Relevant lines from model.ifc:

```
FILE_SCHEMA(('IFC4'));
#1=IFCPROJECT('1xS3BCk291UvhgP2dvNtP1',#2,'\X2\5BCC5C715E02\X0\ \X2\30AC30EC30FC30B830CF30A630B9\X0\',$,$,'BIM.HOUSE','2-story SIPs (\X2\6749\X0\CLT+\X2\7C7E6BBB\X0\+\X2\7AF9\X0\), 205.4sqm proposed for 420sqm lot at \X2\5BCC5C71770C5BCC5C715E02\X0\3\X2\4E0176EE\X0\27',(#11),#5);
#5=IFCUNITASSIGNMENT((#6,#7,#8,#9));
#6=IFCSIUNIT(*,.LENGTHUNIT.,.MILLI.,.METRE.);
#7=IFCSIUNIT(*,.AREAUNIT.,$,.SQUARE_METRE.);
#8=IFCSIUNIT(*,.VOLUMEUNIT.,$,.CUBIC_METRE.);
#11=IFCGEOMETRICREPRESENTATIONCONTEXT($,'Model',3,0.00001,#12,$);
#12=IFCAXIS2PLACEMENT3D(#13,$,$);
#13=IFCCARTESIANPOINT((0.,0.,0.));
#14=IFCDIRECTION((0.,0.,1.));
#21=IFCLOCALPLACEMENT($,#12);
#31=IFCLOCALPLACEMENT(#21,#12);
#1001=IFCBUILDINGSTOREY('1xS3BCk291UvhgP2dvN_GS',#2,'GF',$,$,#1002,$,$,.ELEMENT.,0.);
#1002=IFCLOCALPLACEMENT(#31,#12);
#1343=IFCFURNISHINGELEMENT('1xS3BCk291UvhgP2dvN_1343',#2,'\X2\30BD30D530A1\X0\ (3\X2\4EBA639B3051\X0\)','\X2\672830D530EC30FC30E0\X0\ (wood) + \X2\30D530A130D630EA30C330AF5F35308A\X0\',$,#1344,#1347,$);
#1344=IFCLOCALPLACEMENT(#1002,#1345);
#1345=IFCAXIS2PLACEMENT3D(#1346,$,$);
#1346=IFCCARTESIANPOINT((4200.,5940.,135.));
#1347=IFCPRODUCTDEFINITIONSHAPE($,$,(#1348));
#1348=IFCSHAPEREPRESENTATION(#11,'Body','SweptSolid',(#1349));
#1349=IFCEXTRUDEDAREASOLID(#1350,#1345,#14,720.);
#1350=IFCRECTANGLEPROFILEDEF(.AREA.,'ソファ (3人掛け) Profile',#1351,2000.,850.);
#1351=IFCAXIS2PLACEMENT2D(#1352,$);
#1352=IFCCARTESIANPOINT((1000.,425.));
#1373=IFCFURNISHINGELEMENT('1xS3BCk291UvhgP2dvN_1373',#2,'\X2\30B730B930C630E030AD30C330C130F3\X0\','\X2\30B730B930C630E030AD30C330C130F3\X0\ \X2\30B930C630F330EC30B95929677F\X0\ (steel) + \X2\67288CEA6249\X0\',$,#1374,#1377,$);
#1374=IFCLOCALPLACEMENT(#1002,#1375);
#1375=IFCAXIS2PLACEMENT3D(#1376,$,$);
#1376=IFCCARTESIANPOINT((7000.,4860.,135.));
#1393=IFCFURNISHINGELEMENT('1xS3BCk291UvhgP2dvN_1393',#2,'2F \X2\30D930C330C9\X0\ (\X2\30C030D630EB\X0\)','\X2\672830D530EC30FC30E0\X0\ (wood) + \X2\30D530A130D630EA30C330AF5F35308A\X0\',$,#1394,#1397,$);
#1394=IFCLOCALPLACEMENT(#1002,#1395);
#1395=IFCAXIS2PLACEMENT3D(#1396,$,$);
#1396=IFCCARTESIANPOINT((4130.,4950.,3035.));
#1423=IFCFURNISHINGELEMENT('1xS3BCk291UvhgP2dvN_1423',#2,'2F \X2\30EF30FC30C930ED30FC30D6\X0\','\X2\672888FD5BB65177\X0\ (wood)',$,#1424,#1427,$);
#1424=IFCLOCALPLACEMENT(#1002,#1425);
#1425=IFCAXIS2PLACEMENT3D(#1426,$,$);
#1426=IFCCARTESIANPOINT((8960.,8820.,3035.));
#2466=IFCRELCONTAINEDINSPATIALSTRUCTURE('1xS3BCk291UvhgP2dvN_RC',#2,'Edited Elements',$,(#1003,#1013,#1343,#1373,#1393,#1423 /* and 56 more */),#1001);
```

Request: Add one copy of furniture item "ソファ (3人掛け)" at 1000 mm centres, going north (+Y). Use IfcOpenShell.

```python
import numpy as np
import ifcopenshell
import ifcopenshell.api.geometry
import ifcopenshell.api.root
import ifcopenshell.util.element
import ifcopenshell.util.placement

model = ifcopenshell.open("model.ifc")


def reuse_history(source, copy):
    """copy_class also copies each property set's owner history, people and application; keep the originals."""
    for rel in copy.IsDefinedBy:
        if rel.is_a("IfcRelDefinesByProperties") and (history := rel.RelatingPropertyDefinition.OwnerHistory):
            rel.RelatingPropertyDefinition.OwnerHistory = source.OwnerHistory
            ifcopenshell.util.element.remove_deep2(model, history)


source = model.by_id(1343)
base = ifcopenshell.util.placement.get_local_placement(source.ObjectPlacement)
step = np.array([0.0, 1.0, 0.0]) * 1000.0

for i in range(1, 2):
    copy = ifcopenshell.api.root.copy_class(model, product=source)
    copy.Representation = ifcopenshell.util.element.copy_deep(
        model, source.Representation, exclude=["IfcGeometricRepresentationContext", "IfcRepresentationMap"]
    )
    reuse_history(source, copy)
    matrix = base.copy()
    matrix[:3, 3] += i * step
    print("added at", matrix[:3, 3].round(3) + 0.0)
    ifcopenshell.api.geometry.edit_object_placement(model, product=copy, matrix=matrix, is_si=False)

model.write("model_updated.ifc")
```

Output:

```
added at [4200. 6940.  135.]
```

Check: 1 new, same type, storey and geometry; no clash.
